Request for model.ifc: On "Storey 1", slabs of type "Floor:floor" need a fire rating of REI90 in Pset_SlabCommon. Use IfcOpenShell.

First a look at what the model holds.

```python
import ifcopenshell
import ifcopenshell.util.element

model = ifcopenshell.open("model.ifc")
print(model.schema)
storey = next(s for s in model.by_type("IfcBuildingStorey") if s.Name == "Storey 1")
slabs = [e for e in ifcopenshell.util.element.get_decomposition(storey) if e.is_a("IfcSlab")]
seen = {}
for e in slabs:
    element_type = ifcopenshell.util.element.get_type(e)
    key = (element_type.Name if element_type != e and element_type else None, ifcopenshell.util.element.get_pset(e, "Pset_SlabCommon", "FireRating"))
    seen[key] = seen.get(key, 0) + 1
for (name, value), count in sorted(seen.items(), key=str):
    print(count, "x", name, "|", value)
```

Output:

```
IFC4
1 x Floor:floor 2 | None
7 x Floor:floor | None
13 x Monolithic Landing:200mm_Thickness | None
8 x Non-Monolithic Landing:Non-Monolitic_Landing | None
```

```python
import ifcopenshell
import ifcopenshell.api.pset
import ifcopenshell.util.element

model = ifcopenshell.open("model.ifc")

storey = next(s for s in model.by_type("IfcBuildingStorey") if s.Name == "Storey 1")
slabs = [e for e in ifcopenshell.util.element.get_decomposition(storey) if e.is_a("IfcSlab")]

count = 0
for e in slabs:
    element_type = ifcopenshell.util.element.get_type(e)
    if element_type in (None, e) or element_type.Name != "Floor:floor":
        continue
    # add_pset returns the element's existing set when there is one.
    pset = ifcopenshell.api.pset.add_pset(model, product=e, name="Pset_SlabCommon")
    ifcopenshell.api.pset.edit_pset(model, pset=pset, properties={"FireRating": "REI90"})
    count += 1

print(count, "slabs updated")

model.write("model_updated.ifc")
```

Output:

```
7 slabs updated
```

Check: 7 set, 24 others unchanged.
